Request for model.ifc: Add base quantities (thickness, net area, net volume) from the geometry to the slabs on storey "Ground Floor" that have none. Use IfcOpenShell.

First a look at what the model holds.

```python
import ifcopenshell
import ifcopenshell.util.element
import ifcopenshell.util.unit

model = ifcopenshell.open("model.ifc")
print(model.schema)
for unit_type in ("LENGTHUNIT", "AREAUNIT", "VOLUMEUNIT"):
    print(unit_type, ifcopenshell.util.unit.calculate_unit_scale(model, unit_type))
storey = next(s for s in model.by_type("IfcBuildingStorey") if s.Name == "Ground Floor")
slabs = [e for e in ifcopenshell.util.element.get_decomposition(storey) if e.is_a("IfcSlab")]
for e in sorted(slabs, key=lambda e: e.id()):
    print(e.id(), e.is_a(), e.Name, list(ifcopenshell.util.element.get_psets(e, qtos_only=True)), sep=" | ")
```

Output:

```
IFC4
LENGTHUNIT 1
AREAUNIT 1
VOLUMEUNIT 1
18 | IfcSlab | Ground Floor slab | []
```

```python
import ifcopenshell
import ifcopenshell.api.pset
import ifcopenshell.geom
import ifcopenshell.util.element
import ifcopenshell.util.shape
import ifcopenshell.util.unit

model = ifcopenshell.open("model.ifc")
unit_scale = ifcopenshell.util.unit.calculate_unit_scale(model)
area_scale = ifcopenshell.util.unit.calculate_unit_scale(model, "AREAUNIT")
volume_scale = ifcopenshell.util.unit.calculate_unit_scale(model, "VOLUMEUNIT")
settings = ifcopenshell.geom.settings()

storey = next(s for s in model.by_type("IfcBuildingStorey") if s.Name == "Ground Floor")
slabs = [e for e in ifcopenshell.util.element.get_decomposition(storey) if e.is_a("IfcSlab")]

for e in sorted(slabs, key=lambda e: e.id()):
    if ifcopenshell.util.element.get_psets(e, qtos_only=True, should_inherit=False):
        continue
    # Geometry comes back in metres, in the element's own axes.
    shape = ifcopenshell.geom.create_shape(settings, e)
    values = {
        "Width": ifcopenshell.util.shape.get_z(shape.geometry) / unit_scale,
        "NetArea": ifcopenshell.util.shape.get_footprint_area(shape.geometry) / area_scale,
        "NetVolume": ifcopenshell.util.shape.get_volume(shape.geometry) / volume_scale,
    }
    qto = ifcopenshell.api.pset.add_qto(model, product=e, name="Qto_SlabBaseQuantities")
    ifcopenshell.api.pset.edit_qto(model, qto=qto, properties=values)
    print(e.id(), {k: round(v, 3) for k, v in values.items()})

model.write("model_updated.ifc")
```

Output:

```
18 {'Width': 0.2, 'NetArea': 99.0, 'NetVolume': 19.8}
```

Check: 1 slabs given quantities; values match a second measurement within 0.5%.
